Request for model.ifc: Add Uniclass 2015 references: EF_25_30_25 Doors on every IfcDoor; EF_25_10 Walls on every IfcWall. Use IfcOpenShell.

First a look at what the model holds.

```python
import ifcopenshell

model = ifcopenshell.open("model.ifc")
print(model.schema)
print("classifications:", [c.Name for c in model.by_type("IfcClassification")])
for ifc_class in ("IfcDoor", "IfcRoof", "IfcStair", "IfcWall", "IfcWindow"):
    print(ifc_class, len(model.by_type(ifc_class)))
```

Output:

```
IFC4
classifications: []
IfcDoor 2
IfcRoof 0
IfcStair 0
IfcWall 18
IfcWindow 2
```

```python
import ifcopenshell
import ifcopenshell.api.classification

model = ifcopenshell.open("model.ifc")

system = ifcopenshell.api.classification.add_classification(model, classification="Uniclass 2015")

codes = {
    "IfcDoor": ("EF_25_30_25", "Doors"),
    "IfcWall": ("EF_25_10", "Walls"),
}
for ifc_class, (code, name) in codes.items():
    products = model.by_type(ifc_class)
    ifcopenshell.api.classification.add_reference(
        model, products=products, classification=system, identification=code, name=name
    )
    print(code, len(products))

model.write("model-out.ifc")
```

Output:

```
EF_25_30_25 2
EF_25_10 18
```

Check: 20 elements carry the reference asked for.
